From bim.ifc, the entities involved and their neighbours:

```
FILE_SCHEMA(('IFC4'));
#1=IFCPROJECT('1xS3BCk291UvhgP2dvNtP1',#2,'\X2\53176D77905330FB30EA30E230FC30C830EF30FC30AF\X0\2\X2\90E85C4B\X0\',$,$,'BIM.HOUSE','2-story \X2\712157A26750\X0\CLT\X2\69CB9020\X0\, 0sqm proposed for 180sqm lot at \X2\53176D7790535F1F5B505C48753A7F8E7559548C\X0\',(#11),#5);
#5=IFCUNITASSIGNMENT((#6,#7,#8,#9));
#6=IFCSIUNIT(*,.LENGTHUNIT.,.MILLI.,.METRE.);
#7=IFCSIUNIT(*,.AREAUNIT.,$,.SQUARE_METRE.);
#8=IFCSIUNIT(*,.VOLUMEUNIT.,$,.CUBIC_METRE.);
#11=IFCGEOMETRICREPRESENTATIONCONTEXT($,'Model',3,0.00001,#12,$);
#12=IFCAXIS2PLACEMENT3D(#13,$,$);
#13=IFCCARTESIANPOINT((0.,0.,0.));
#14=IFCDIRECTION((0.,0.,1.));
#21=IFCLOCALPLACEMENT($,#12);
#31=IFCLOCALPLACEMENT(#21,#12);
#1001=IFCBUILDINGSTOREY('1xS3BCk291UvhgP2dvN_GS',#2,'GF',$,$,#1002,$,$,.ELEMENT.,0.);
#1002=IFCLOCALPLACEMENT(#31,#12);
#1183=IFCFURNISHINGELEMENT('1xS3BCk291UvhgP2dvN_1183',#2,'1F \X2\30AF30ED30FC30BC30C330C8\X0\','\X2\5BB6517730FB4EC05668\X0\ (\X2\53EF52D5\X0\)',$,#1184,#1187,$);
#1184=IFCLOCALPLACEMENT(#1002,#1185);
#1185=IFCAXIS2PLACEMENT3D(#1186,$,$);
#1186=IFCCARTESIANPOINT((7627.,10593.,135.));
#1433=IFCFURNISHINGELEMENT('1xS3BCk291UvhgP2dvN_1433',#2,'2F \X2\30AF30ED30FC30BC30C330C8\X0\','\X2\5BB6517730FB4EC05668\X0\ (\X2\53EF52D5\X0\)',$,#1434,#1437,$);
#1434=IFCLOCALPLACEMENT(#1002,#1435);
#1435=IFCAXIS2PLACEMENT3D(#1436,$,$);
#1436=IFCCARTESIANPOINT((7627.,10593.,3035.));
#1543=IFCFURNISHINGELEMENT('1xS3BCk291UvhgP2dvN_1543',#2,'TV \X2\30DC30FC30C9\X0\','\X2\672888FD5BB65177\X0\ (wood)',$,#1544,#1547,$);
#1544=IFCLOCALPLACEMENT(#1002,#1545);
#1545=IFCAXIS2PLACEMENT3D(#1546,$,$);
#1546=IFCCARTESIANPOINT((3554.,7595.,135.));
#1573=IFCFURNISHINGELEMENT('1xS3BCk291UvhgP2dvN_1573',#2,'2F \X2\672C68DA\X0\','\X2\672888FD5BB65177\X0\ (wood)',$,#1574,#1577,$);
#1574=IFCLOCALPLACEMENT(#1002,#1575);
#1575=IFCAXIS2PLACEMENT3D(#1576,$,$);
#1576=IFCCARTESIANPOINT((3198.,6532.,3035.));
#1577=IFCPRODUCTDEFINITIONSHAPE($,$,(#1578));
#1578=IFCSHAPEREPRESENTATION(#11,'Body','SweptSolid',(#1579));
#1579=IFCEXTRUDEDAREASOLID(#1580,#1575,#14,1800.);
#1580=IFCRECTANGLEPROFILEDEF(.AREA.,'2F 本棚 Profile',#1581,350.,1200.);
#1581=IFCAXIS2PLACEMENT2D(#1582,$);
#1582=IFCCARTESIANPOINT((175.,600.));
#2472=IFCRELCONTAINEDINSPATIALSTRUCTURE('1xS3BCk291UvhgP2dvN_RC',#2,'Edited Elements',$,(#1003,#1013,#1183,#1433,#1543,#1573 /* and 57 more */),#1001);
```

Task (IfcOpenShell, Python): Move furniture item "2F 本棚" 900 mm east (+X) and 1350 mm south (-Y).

```python
import ifcopenshell
import ifcopenshell.api.geometry
import ifcopenshell.util.placement

model = ifcopenshell.open("bim.ifc")

item = model.by_guid("1xS3BCk291UvhgP2dvN_1573")
matrix = ifcopenshell.util.placement.get_local_placement(item.ObjectPlacement)
matrix[0, 3] += 900.0
matrix[1, 3] -= 1350.0
ifcopenshell.api.geometry.edit_object_placement(model, product=item, matrix=matrix, is_si=False)

print(ifcopenshell.util.placement.get_local_placement(item.ObjectPlacement).round(3) + 0.0)

model.write("bim_updated.ifc")
```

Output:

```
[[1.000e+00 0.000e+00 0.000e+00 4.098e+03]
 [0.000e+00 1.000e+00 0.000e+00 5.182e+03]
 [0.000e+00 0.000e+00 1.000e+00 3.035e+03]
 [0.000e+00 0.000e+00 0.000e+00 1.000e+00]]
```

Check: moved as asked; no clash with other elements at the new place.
